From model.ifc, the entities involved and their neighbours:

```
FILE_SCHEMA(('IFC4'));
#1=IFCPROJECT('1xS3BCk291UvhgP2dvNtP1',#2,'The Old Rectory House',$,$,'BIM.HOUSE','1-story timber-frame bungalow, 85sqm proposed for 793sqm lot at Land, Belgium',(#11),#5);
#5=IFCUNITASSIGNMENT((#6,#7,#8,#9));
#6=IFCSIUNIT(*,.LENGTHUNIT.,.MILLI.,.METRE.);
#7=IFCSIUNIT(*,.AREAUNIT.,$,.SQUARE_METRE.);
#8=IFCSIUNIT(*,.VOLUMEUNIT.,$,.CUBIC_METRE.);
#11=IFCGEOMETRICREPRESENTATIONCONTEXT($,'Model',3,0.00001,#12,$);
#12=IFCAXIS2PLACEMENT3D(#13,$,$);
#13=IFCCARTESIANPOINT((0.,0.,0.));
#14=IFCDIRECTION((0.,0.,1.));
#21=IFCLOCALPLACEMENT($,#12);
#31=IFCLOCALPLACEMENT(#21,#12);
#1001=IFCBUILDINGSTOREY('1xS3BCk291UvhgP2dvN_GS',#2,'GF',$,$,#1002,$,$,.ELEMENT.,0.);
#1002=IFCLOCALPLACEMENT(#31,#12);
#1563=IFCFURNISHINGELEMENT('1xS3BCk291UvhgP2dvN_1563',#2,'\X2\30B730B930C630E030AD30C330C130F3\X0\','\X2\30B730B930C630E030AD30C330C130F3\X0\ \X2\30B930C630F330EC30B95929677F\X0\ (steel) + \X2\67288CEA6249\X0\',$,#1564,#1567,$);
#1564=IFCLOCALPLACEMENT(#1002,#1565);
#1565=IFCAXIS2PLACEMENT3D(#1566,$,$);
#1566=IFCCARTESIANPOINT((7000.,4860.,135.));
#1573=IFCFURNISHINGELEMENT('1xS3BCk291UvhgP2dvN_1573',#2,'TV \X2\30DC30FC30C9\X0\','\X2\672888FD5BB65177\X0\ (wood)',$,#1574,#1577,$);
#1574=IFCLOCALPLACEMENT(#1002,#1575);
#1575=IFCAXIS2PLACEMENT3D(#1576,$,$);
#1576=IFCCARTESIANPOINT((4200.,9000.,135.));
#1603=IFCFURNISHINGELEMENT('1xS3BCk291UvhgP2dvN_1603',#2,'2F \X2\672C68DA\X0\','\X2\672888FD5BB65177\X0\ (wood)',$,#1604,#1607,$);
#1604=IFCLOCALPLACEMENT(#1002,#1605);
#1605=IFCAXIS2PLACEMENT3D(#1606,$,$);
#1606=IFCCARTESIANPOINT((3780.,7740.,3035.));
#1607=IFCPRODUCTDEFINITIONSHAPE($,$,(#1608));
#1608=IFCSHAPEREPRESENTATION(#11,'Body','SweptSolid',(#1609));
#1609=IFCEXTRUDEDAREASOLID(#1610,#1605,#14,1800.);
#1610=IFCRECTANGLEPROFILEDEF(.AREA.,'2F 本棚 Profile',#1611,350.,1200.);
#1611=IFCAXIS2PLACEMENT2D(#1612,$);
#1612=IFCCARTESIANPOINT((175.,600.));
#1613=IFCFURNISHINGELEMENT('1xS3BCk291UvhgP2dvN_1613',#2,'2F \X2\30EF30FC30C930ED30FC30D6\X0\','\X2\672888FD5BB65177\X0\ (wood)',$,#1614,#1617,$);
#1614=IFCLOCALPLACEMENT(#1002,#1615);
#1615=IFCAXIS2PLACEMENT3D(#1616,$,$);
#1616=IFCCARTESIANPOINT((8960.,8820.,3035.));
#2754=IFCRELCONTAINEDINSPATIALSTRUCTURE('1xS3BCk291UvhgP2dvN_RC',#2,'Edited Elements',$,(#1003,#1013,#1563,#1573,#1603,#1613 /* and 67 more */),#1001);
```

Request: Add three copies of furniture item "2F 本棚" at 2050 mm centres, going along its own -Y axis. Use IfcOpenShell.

```python
import ifcopenshell
import ifcopenshell.api.geometry
import ifcopenshell.api.root
import ifcopenshell.util.element
import ifcopenshell.util.placement

model = ifcopenshell.open("model.ifc")


def reuse_history(source, copy):
    """copy_class also copies each property set's owner history, people and application; keep the originals."""
    for rel in copy.IsDefinedBy:
        if rel.is_a("IfcRelDefinesByProperties") and (history := rel.RelatingPropertyDefinition.OwnerHistory):
            rel.RelatingPropertyDefinition.OwnerHistory = source.OwnerHistory
            ifcopenshell.util.element.remove_deep2(model, history)


source = model.by_guid("1xS3BCk291UvhgP2dvN_1603")
base = ifcopenshell.util.placement.get_local_placement(source.ObjectPlacement)
step = -base[:3, 1] * 2050.0

for i in range(1, 4):
    copy = ifcopenshell.api.root.copy_class(model, product=source)
    copy.Representation = ifcopenshell.util.element.copy_deep(
        model, source.Representation, exclude=["IfcGeometricRepresentationContext", "IfcRepresentationMap"]
    )
    reuse_history(source, copy)
    matrix = base.copy()
    matrix[:3, 3] += i * step
    print("added at", matrix[:3, 3].round(3) + 0.0)
    ifcopenshell.api.geometry.edit_object_placement(model, product=copy, matrix=matrix, is_si=False)

model.write("model_rev.ifc")
```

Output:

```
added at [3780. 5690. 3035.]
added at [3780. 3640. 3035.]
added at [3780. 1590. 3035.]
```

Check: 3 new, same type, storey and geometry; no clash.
